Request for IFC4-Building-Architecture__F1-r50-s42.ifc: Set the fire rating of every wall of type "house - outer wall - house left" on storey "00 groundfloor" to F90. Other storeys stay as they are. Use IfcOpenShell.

First a look at what the model holds.

```python
import ifcopenshell
import ifcopenshell.util.element

model = ifcopenshell.open("IFC4-Building-Architecture__F1-r50-s42.ifc")
print(model.schema)
storey = next(s for s in model.by_type("IfcBuildingStorey") if s.Name == "00 groundfloor")
walls = [e for e in ifcopenshell.util.element.get_decomposition(storey) if e.is_a("IfcWall")]
seen = {}
for e in walls:
    element_type = ifcopenshell.util.element.get_type(e)
    key = (element_type.Name if element_type != e and element_type else None, ifcopenshell.util.element.get_pset(e, "Pset_WallCommon", "FireRating"))
    seen[key] = seen.get(key, 0) + 1
for (name, value), count in sorted(seen.items(), key=str):
    print(count, "x", name, "|", value)
```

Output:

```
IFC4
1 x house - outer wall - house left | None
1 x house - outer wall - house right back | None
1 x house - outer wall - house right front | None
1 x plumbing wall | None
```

```python
import ifcopenshell
import ifcopenshell.api.pset
import ifcopenshell.util.element

model = ifcopenshell.open("IFC4-Building-Architecture__F1-r50-s42.ifc")

storey = next(s for s in model.by_type("IfcBuildingStorey") if s.Name == "00 groundfloor")
walls = [e for e in ifcopenshell.util.element.get_decomposition(storey) if e.is_a("IfcWall")]

count = 0
for e in walls:
    element_type = ifcopenshell.util.element.get_type(e)
    if element_type in (None, e) or element_type.Name != "house - outer wall - house left":
        continue
    # add_pset returns the element's existing set when there is one.
    pset = ifcopenshell.api.pset.add_pset(model, product=e, name="Pset_WallCommon")
    ifcopenshell.api.pset.edit_pset(model, pset=pset, properties={"FireRating": "F90"})
    count += 1

print(count, "walls updated")

model.write("IFC4-Building-Architecture__F1-r50-s42_v2.ifc")
```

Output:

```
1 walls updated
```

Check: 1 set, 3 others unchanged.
